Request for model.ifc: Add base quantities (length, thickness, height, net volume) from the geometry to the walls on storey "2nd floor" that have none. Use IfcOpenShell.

First a look at what the model holds.

```python
import ifcopenshell
import ifcopenshell.util.element
import ifcopenshell.util.unit

model = ifcopenshell.open("model.ifc")
print(model.schema)
for unit_type in ("LENGTHUNIT", "AREAUNIT", "VOLUMEUNIT"):
    print(unit_type, ifcopenshell.util.unit.calculate_unit_scale(model, unit_type))
storey = next(s for s in model.by_type("IfcBuildingStorey") if s.Name == "2nd floor")
walls = [e for e in ifcopenshell.util.element.get_decomposition(storey) if e.is_a("IfcWall")]
for e in sorted(walls, key=lambda e: e.id()):
    print(e.id(), e.is_a(), e.Name, list(ifcopenshell.util.element.get_psets(e, qtos_only=True)), sep=" | ")
```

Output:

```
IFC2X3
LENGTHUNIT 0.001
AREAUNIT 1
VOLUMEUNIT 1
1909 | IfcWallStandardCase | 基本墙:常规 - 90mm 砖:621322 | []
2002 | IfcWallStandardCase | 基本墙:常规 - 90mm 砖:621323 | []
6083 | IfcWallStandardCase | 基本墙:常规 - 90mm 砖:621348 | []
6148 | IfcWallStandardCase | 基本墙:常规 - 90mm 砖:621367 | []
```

```python
import ifcopenshell
import ifcopenshell.api.pset
import ifcopenshell.geom
import ifcopenshell.util.element
import ifcopenshell.util.shape
import ifcopenshell.util.unit

model = ifcopenshell.open("model.ifc")
unit_scale = ifcopenshell.util.unit.calculate_unit_scale(model)
volume_scale = ifcopenshell.util.unit.calculate_unit_scale(model, "VOLUMEUNIT")
settings = ifcopenshell.geom.settings()

storey = next(s for s in model.by_type("IfcBuildingStorey") if s.Name == "2nd floor")
walls = [e for e in ifcopenshell.util.element.get_decomposition(storey) if e.is_a("IfcWall")]

for e in sorted(walls, key=lambda e: e.id()):
    if ifcopenshell.util.element.get_psets(e, qtos_only=True, should_inherit=False):
        continue
    # Geometry comes back in metres, in the element's own axes.
    shape = ifcopenshell.geom.create_shape(settings, e)
    values = {
        "Length": ifcopenshell.util.shape.get_x(shape.geometry) / unit_scale,
        "Width": ifcopenshell.util.shape.get_y(shape.geometry) / unit_scale,
        "Height": ifcopenshell.util.shape.get_z(shape.geometry) / unit_scale,
        "NetVolume": ifcopenshell.util.shape.get_volume(shape.geometry) / volume_scale,
    }
    qto = ifcopenshell.api.pset.add_qto(model, product=e, name="BaseQuantities")
    ifcopenshell.api.pset.edit_qto(model, qto=qto, properties=values)
    print(e.id(), {k: round(v, 3) for k, v in values.items()})

model.write("model_updated.ifc")
```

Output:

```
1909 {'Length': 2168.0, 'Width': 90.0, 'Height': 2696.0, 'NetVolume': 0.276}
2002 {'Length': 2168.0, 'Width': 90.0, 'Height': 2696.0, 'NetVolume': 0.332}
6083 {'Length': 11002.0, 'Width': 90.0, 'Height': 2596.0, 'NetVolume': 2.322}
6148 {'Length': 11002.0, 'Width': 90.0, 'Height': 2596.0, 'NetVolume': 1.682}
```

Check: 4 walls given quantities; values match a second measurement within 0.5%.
